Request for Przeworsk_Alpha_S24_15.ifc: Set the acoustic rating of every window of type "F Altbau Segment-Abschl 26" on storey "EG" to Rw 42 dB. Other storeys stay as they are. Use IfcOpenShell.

First a look at what the model holds.

```python
import ifcopenshell
import ifcopenshell.util.element

model = ifcopenshell.open("Przeworsk_Alpha_S24_15.ifc")
print(model.schema)
storey = next(s for s in model.by_type("IfcBuildingStorey") if s.Name == "EG")
windows = [e for e in ifcopenshell.util.element.get_decomposition(storey) if e.is_a("IfcWindow")]
seen = {}
for e in windows:
    element_type = ifcopenshell.util.element.get_type(e)
    key = (element_type.Name if element_type != e and element_type else None, ifcopenshell.util.element.get_pset(e, "Pset_WindowCommon", "AcousticRating"))
    seen[key] = seen.get(key, 0) + 1
for (name, value), count in sorted(seen.items(), key=str):
    print(count, "x", name, "|", value)
```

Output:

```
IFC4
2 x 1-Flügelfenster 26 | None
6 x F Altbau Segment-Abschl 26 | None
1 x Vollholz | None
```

```python
import ifcopenshell
import ifcopenshell.api.pset
import ifcopenshell.util.element

model = ifcopenshell.open("Przeworsk_Alpha_S24_15.ifc")

storey = next(s for s in model.by_type("IfcBuildingStorey") if s.Name == "EG")
windows = [e for e in ifcopenshell.util.element.get_decomposition(storey) if e.is_a("IfcWindow")]

count = 0
for e in windows:
    element_type = ifcopenshell.util.element.get_type(e)
    if element_type in (None, e) or element_type.Name != "F Altbau Segment-Abschl 26":
        continue
    # add_pset returns the element's existing set when there is one.
    pset = ifcopenshell.api.pset.add_pset(model, product=e, name="Pset_WindowCommon")
    ifcopenshell.api.pset.edit_pset(model, pset=pset, properties={"AcousticRating": "Rw 42 dB"})
    count += 1

print(count, "windows updated")

model.write("Przeworsk_Alpha_S24_15_rev.ifc")
```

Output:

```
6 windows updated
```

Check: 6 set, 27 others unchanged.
